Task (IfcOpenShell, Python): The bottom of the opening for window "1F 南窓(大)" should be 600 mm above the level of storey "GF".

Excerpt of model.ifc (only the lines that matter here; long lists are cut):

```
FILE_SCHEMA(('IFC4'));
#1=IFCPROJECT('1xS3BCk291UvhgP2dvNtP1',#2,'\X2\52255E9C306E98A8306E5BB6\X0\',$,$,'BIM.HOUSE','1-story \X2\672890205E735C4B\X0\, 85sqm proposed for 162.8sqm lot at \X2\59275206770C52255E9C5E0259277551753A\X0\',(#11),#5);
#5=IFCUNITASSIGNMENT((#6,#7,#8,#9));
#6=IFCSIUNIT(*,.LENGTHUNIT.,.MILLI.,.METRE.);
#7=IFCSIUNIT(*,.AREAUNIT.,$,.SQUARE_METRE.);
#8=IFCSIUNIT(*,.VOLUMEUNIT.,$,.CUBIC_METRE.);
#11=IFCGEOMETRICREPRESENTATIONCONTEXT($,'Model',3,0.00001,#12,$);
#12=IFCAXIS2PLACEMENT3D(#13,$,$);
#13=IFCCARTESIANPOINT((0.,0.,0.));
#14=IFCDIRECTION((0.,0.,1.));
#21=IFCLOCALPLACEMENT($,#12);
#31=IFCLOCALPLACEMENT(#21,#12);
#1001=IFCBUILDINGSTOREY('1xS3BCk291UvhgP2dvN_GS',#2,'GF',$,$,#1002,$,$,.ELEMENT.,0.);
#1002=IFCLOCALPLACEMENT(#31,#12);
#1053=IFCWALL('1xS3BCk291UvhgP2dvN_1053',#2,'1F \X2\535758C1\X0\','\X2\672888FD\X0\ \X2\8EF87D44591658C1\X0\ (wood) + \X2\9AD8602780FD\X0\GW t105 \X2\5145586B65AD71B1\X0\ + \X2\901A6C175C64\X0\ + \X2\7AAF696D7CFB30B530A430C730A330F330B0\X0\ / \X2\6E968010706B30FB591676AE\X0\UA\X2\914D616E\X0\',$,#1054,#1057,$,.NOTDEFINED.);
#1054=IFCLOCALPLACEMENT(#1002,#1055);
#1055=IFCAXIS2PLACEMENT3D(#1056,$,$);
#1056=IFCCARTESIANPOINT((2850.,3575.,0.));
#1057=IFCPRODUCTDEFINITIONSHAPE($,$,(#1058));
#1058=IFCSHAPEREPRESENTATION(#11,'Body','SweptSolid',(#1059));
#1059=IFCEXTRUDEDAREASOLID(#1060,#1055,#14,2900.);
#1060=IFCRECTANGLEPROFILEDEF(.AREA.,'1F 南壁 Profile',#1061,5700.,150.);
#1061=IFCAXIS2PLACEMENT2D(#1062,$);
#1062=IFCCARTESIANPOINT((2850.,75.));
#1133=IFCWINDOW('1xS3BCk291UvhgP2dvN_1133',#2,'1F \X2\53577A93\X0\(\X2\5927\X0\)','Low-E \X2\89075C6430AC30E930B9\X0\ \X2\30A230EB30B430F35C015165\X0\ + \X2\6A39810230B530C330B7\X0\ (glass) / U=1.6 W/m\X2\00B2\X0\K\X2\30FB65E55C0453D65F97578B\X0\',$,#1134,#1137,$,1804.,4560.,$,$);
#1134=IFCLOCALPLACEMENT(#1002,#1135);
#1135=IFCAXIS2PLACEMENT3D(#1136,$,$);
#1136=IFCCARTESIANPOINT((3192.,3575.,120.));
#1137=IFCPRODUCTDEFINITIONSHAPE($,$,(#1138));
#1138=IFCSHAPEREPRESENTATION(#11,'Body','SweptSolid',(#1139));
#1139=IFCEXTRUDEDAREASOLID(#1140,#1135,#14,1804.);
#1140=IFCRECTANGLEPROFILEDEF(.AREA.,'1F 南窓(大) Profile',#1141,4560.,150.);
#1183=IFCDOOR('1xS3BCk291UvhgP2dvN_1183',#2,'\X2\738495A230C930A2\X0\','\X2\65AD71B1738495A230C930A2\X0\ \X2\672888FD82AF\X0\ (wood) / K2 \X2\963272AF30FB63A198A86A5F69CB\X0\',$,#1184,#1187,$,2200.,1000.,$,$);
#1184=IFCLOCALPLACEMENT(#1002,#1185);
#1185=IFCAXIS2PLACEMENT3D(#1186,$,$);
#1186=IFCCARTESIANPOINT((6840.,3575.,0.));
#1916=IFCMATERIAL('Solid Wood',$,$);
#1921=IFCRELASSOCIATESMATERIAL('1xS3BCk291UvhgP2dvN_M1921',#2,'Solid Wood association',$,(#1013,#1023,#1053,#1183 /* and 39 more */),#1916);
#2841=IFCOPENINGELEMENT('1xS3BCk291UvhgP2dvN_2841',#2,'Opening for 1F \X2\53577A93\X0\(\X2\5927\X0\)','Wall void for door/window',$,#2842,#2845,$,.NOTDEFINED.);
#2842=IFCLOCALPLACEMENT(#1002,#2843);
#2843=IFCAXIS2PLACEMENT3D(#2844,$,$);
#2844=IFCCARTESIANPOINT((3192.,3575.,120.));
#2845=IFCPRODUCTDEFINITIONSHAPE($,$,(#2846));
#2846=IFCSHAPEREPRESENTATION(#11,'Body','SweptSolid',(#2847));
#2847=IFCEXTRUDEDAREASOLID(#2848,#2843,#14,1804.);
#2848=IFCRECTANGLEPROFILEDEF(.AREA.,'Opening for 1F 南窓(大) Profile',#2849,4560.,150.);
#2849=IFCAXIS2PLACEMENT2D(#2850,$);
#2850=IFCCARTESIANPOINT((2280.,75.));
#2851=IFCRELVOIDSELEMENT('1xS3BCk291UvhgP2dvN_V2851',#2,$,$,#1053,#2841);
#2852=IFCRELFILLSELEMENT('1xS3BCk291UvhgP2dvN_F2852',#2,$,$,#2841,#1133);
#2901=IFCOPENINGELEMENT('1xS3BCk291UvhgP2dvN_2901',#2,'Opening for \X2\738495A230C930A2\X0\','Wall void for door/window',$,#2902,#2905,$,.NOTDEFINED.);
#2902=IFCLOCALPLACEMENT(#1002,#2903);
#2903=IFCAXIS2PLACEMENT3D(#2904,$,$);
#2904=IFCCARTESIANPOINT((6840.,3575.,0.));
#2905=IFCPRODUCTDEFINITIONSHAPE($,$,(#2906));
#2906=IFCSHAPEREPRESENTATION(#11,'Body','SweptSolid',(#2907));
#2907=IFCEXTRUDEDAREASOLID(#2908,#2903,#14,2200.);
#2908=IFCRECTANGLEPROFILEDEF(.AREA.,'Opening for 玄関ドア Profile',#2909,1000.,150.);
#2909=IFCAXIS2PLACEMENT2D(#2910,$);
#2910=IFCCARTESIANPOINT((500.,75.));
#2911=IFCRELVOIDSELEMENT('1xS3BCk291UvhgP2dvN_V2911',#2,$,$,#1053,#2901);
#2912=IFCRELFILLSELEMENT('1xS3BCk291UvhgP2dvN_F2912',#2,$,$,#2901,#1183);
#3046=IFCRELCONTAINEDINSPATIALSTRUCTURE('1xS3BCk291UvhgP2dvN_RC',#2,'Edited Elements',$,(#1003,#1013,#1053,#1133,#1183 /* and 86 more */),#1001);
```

```python
import numpy as np
import ifcopenshell
import ifcopenshell.api.geometry
import ifcopenshell.geom
import ifcopenshell.util.element
import ifcopenshell.util.placement
import ifcopenshell.util.shape
import ifcopenshell.util.unit

model = ifcopenshell.open("model.ifc")
unit_scale = ifcopenshell.util.unit.calculate_unit_scale(model)

window = model.by_guid("1xS3BCk291UvhgP2dvN_1133")
opening = window.FillsVoids[0].RelatingOpeningElement
storey = ifcopenshell.util.element.get_container(window, ifc_class="IfcBuildingStorey")
level = ifcopenshell.util.placement.get_local_placement(storey.ObjectPlacement)[2, 3]

# The opening's origin need not be at the sill, so measure its lowest point.
shape = ifcopenshell.geom.create_shape(ifcopenshell.geom.settings(), opening)
bottom = ifcopenshell.util.shape.get_shape_bottom_elevation(shape, shape.geometry) / unit_scale
dz = level + 0.6 / unit_scale - bottom

shift = np.array([0.0, 0.0, dz])
# The window is not placed relative to its opening, so move both.
for product in (opening, window):
    matrix = ifcopenshell.util.placement.get_local_placement(product.ObjectPlacement)
    matrix[:3, 3] += shift
    ifcopenshell.api.geometry.edit_object_placement(model, product=product, matrix=matrix, is_si=False)

print(f"moved by {dz * unit_scale:+.3f} m")

model.write("model-out.ifc")
```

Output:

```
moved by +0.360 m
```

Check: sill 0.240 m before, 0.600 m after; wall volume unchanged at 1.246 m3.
